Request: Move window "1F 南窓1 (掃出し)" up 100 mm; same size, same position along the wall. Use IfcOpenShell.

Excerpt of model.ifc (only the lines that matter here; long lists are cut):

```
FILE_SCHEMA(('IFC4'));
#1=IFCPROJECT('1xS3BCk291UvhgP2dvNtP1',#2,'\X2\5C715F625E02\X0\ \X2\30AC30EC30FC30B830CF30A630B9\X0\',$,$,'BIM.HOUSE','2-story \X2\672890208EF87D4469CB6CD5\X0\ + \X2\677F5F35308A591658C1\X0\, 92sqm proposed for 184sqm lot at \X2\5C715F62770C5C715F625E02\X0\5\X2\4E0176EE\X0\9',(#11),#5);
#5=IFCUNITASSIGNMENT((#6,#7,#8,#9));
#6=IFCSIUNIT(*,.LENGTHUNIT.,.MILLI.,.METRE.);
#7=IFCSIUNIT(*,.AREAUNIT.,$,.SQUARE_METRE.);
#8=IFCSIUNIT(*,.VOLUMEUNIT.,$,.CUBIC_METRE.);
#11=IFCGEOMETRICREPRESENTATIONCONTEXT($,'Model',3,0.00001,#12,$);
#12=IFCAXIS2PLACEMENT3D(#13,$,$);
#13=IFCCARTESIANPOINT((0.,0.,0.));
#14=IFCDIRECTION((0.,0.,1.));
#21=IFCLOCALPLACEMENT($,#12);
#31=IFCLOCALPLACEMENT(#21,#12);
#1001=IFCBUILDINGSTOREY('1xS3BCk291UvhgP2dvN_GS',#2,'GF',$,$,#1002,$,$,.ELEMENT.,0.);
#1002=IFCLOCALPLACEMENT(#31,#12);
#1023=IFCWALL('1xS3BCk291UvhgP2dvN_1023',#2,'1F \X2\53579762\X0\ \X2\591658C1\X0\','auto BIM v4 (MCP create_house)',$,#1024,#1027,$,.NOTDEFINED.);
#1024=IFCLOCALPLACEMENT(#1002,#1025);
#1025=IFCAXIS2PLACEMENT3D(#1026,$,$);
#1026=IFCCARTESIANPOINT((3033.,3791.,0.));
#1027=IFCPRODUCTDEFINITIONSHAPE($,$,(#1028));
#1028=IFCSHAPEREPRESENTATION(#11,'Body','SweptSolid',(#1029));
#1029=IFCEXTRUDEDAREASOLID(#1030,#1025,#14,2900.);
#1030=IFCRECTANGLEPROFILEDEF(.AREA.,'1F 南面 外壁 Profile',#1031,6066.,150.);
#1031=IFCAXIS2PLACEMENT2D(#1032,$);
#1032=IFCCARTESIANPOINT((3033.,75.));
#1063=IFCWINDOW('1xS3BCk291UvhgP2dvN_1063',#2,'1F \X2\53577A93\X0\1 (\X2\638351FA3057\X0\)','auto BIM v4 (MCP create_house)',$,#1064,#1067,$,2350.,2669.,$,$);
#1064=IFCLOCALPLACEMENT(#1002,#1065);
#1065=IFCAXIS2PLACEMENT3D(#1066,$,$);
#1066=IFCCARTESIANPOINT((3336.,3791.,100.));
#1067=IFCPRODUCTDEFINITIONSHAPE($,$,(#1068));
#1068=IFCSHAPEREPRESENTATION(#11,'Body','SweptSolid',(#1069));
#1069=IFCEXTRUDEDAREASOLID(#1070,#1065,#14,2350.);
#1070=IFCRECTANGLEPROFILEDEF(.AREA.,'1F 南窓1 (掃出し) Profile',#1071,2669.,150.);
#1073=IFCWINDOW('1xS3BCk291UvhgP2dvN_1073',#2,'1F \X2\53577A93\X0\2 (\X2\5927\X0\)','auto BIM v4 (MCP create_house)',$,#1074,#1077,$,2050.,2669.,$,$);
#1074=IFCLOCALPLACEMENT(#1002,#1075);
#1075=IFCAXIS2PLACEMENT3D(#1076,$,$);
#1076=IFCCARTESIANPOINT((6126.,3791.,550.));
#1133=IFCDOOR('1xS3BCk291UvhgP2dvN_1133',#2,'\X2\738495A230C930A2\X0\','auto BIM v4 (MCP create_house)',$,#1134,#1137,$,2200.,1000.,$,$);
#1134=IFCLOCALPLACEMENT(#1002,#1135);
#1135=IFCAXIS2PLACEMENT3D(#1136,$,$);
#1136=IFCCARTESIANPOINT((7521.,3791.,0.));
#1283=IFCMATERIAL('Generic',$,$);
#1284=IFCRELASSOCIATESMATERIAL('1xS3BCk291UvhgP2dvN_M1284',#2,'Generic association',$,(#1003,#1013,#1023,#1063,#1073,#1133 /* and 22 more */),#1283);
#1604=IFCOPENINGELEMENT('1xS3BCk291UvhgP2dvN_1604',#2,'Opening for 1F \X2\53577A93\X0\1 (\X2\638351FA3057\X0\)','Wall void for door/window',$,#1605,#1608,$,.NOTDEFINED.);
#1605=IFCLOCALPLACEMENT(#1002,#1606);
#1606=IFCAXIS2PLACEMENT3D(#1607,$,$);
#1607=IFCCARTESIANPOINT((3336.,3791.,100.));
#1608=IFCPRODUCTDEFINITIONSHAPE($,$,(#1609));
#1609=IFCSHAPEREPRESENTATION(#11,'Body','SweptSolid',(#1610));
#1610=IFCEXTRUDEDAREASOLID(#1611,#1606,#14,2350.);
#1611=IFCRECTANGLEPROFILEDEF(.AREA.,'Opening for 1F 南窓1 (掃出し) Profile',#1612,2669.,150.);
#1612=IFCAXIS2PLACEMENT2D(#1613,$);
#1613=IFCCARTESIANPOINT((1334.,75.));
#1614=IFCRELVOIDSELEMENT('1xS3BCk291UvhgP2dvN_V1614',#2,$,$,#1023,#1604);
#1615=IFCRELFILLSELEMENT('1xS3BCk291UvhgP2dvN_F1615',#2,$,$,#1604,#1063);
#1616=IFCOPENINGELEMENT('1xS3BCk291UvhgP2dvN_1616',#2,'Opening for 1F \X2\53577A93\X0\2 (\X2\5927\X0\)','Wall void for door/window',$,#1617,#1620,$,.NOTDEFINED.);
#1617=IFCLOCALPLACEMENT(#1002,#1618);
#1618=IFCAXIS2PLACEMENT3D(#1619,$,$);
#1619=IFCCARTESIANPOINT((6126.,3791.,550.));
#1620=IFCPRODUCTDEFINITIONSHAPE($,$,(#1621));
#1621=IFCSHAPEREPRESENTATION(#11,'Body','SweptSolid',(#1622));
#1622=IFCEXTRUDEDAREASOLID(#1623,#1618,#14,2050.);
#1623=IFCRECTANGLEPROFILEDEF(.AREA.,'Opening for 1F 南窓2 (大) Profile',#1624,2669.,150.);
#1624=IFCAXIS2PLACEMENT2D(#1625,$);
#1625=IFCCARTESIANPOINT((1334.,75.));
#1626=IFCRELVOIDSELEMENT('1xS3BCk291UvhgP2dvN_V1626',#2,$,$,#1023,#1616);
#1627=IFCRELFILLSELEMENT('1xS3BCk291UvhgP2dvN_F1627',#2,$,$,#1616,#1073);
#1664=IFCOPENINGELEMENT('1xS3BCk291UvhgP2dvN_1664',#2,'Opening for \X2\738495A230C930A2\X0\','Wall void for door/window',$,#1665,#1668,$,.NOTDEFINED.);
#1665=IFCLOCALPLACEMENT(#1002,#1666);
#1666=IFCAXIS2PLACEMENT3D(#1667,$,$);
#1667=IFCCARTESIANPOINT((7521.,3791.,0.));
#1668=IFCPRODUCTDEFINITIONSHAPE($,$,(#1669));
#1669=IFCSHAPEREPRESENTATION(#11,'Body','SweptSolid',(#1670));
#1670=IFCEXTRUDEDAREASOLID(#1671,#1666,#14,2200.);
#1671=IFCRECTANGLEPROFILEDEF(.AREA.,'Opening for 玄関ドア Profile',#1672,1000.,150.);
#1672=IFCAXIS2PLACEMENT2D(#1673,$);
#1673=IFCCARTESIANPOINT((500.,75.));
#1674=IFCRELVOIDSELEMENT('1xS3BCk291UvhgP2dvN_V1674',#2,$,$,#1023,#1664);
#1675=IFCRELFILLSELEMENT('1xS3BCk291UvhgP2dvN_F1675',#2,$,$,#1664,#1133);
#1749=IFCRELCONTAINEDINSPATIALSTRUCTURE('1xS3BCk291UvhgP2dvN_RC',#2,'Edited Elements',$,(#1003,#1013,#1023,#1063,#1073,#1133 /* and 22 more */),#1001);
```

```python
import numpy as np
import ifcopenshell
import ifcopenshell.api.geometry
import ifcopenshell.util.placement
import ifcopenshell.util.unit

model = ifcopenshell.open("model.ifc")
unit_scale = ifcopenshell.util.unit.calculate_unit_scale(model)

window = model.by_guid("1xS3BCk291UvhgP2dvN_1063")
opening = window.FillsVoids[0].RelatingOpeningElement
dz = 100.0

shift = np.array([0.0, 0.0, dz])
# The window is not placed relative to its opening, so move both.
for product in (opening, window):
    matrix = ifcopenshell.util.placement.get_local_placement(product.ObjectPlacement)
    matrix[:3, 3] += shift
    ifcopenshell.api.geometry.edit_object_placement(model, product=product, matrix=matrix, is_si=False)

print(f"moved by {dz * unit_scale:+.3f} m")

model.write("model_v2.ifc")
```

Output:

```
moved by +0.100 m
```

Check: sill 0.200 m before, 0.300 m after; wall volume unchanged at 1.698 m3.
